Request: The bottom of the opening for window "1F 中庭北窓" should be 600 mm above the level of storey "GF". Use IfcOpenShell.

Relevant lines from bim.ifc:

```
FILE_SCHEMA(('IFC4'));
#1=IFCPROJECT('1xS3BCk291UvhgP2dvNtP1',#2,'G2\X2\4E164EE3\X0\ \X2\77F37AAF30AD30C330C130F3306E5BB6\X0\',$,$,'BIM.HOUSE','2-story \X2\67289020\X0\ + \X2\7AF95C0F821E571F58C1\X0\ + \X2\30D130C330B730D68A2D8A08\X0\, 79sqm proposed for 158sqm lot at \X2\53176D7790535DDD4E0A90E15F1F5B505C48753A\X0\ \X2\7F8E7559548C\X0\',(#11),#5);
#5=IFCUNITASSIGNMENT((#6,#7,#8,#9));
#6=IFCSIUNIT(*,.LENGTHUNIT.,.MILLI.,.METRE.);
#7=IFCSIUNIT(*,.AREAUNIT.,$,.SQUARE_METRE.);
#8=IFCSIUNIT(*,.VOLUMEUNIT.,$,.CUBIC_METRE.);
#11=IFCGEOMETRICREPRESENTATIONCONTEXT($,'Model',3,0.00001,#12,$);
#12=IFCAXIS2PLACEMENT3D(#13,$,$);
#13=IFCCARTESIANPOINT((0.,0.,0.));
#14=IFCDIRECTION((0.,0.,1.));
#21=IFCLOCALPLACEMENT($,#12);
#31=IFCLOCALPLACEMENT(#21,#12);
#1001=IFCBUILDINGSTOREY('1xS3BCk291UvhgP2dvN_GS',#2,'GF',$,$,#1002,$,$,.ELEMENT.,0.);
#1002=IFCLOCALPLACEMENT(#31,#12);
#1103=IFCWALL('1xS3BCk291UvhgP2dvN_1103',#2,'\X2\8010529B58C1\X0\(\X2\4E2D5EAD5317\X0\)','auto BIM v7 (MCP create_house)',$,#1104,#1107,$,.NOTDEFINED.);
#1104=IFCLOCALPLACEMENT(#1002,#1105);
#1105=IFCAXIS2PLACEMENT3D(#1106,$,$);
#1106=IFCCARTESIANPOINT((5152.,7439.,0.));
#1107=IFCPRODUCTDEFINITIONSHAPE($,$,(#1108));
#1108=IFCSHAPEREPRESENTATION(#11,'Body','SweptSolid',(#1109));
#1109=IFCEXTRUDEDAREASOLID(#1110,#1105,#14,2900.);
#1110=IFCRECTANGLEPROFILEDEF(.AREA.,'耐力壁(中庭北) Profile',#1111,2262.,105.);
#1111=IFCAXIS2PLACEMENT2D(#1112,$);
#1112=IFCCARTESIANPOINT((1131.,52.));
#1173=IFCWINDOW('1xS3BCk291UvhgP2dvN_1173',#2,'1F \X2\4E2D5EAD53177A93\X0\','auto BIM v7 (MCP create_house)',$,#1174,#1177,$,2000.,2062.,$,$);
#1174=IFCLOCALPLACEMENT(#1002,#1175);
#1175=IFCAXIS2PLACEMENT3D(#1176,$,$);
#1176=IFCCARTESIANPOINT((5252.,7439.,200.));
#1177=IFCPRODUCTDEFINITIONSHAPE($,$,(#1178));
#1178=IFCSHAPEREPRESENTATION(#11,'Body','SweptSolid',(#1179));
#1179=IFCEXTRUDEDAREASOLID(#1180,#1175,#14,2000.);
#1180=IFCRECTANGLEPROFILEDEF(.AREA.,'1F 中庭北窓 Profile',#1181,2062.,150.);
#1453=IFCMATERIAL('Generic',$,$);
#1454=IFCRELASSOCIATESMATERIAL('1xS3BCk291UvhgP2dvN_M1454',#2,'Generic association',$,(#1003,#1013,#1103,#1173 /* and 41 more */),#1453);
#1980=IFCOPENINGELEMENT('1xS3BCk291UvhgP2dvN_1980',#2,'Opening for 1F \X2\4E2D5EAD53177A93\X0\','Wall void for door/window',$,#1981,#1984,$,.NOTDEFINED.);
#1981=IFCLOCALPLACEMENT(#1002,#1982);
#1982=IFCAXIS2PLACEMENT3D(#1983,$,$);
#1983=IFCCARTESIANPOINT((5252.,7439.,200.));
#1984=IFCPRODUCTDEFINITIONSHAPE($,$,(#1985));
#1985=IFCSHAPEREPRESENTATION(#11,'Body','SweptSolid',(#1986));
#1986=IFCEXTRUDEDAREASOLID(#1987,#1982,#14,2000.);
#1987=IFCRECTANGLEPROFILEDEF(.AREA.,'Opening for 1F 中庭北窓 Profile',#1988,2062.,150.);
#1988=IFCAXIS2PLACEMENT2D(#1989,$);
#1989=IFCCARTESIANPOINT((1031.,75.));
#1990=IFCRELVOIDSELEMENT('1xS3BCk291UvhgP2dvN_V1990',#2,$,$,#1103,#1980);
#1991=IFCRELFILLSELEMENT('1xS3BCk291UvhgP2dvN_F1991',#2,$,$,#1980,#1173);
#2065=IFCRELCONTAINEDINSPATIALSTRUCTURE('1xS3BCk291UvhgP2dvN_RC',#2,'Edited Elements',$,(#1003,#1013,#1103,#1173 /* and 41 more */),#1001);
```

```python
import numpy as np
import ifcopenshell
import ifcopenshell.api.geometry
import ifcopenshell.geom
import ifcopenshell.util.element
import ifcopenshell.util.placement
import ifcopenshell.util.shape
import ifcopenshell.util.unit

model = ifcopenshell.open("bim.ifc")
unit_scale = ifcopenshell.util.unit.calculate_unit_scale(model)

window = model.by_guid("1xS3BCk291UvhgP2dvN_1173")
opening = window.FillsVoids[0].RelatingOpeningElement
storey = ifcopenshell.util.element.get_container(window, ifc_class="IfcBuildingStorey")
level = ifcopenshell.util.placement.get_local_placement(storey.ObjectPlacement)[2, 3]

# The opening's origin need not be at the sill, so measure its lowest point.
shape = ifcopenshell.geom.create_shape(ifcopenshell.geom.settings(), opening)
bottom = ifcopenshell.util.shape.get_shape_bottom_elevation(shape, shape.geometry) / unit_scale
dz = level + 0.6 / unit_scale - bottom

shift = np.array([0.0, 0.0, dz])
# The window is not placed relative to its opening, so move both.
for product in (opening, window):
    matrix = ifcopenshell.util.placement.get_local_placement(product.ObjectPlacement)
    matrix[:3, 3] += shift
    ifcopenshell.api.geometry.edit_object_placement(model, product=product, matrix=matrix, is_si=False)

print(f"moved by {dz * unit_scale:+.3f} m")

model.write("bim_rev.ifc")
```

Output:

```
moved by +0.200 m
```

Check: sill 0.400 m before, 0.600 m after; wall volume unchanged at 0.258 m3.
